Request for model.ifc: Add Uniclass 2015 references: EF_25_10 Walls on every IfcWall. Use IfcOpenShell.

First a look at what the model holds.

```python
import ifcopenshell

model = ifcopenshell.open("model.ifc")
print(model.schema)
print("classifications:", [c.Name for c in model.by_type("IfcClassification")])
for ifc_class in ("IfcDoor", "IfcRoof", "IfcStair", "IfcWall", "IfcWindow"):
    print(ifc_class, len(model.by_type(ifc_class)))
```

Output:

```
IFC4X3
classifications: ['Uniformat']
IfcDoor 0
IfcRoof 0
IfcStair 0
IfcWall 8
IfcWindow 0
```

```python
import ifcopenshell
import ifcopenshell.api.classification

model = ifcopenshell.open("model.ifc")

system = ifcopenshell.api.classification.add_classification(model, classification="Uniclass 2015")

codes = {
    "IfcWall": ("EF_25_10", "Walls"),
}
for ifc_class, (code, name) in codes.items():
    products = model.by_type(ifc_class)
    ifcopenshell.api.classification.add_reference(
        model, products=products, classification=system, identification=code, name=name
    )
    print(code, len(products))

model.write("model-out.ifc")
```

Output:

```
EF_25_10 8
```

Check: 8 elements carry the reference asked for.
